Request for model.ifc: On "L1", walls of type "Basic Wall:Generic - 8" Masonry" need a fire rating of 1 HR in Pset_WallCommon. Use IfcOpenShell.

First a look at what the model holds.

```python
import ifcopenshell
import ifcopenshell.util.element

model = ifcopenshell.open("model.ifc")
print(model.schema)
storey = next(s for s in model.by_type("IfcBuildingStorey") if s.Name == "L1")
walls = [e for e in ifcopenshell.util.element.get_decomposition(storey) if e.is_a("IfcWall")]
seen = {}
for e in walls:
    element_type = ifcopenshell.util.element.get_type(e)
    key = (element_type.Name if element_type != e and element_type else None, ifcopenshell.util.element.get_pset(e, "Pset_WallCommon", "FireRating"))
    seen[key] = seen.get(key, 0) + 1
for (name, value), count in sorted(seen.items(), key=str):
    print(count, "x", name, "|", value)
```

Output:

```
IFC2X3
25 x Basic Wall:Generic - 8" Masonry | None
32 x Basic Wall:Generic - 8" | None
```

```python
import ifcopenshell
import ifcopenshell.api.pset
import ifcopenshell.util.element

model = ifcopenshell.open("model.ifc")

storey = next(s for s in model.by_type("IfcBuildingStorey") if s.Name == "L1")
walls = [e for e in ifcopenshell.util.element.get_decomposition(storey) if e.is_a("IfcWall")]

count = 0
for e in walls:
    element_type = ifcopenshell.util.element.get_type(e)
    if element_type in (None, e) or element_type.Name != 'Basic Wall:Generic - 8" Masonry':
        continue
    # add_pset returns the element's existing set when there is one.
    pset = ifcopenshell.api.pset.add_pset(model, product=e, name="Pset_WallCommon")
    ifcopenshell.api.pset.edit_pset(model, pset=pset, properties={"FireRating": "1 HR"})
    count += 1

print(count, "walls updated")

model.write("model_rev.ifc")
```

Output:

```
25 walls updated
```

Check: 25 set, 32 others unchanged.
